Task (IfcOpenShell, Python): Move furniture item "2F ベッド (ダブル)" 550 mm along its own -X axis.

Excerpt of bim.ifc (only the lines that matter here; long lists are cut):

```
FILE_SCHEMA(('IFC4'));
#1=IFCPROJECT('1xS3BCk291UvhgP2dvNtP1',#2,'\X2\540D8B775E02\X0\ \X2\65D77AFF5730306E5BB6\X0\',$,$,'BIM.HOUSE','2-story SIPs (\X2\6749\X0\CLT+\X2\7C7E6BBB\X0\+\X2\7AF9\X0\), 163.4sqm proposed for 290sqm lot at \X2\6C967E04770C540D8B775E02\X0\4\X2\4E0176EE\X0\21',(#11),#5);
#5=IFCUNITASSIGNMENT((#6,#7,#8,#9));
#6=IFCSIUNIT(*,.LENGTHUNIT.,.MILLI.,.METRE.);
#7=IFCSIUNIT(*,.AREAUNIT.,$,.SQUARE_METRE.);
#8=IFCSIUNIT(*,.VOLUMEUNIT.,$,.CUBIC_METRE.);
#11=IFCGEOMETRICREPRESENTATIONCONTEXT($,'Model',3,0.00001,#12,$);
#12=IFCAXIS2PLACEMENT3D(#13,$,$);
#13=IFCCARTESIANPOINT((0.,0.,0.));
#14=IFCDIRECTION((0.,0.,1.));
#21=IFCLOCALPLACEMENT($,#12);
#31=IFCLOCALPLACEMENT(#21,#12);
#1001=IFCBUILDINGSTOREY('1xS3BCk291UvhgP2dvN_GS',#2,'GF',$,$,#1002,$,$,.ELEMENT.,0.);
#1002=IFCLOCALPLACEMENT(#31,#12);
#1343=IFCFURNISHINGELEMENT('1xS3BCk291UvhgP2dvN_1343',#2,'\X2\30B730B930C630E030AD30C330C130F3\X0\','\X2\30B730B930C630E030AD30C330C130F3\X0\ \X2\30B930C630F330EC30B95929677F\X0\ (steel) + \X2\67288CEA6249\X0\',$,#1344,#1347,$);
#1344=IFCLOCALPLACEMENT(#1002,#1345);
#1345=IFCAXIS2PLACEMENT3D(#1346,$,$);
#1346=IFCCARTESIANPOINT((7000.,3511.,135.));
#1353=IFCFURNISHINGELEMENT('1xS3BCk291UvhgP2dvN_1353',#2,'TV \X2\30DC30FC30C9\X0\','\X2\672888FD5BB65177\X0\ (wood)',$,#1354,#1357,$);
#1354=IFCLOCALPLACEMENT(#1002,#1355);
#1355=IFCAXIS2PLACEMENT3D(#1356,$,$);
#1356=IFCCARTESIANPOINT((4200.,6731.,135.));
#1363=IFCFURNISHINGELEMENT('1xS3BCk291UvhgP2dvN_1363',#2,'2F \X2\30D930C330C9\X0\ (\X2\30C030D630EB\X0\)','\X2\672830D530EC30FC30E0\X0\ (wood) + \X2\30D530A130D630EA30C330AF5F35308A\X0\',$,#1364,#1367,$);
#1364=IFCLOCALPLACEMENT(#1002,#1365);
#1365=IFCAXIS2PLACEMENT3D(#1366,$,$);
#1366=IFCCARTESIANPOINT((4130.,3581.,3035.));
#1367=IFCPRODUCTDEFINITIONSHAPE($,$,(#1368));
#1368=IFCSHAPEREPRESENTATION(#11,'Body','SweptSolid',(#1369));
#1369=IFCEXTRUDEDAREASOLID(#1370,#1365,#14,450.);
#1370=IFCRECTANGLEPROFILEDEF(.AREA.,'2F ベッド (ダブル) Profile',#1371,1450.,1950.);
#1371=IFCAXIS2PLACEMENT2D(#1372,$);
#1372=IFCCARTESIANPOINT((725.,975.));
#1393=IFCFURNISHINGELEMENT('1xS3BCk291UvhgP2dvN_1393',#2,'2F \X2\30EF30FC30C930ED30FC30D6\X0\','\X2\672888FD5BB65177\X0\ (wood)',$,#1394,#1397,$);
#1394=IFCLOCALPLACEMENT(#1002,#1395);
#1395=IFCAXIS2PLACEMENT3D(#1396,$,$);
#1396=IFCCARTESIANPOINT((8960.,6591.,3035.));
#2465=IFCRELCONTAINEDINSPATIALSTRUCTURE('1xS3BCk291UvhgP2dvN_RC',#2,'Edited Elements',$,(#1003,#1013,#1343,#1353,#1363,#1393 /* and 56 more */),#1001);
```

```python
import ifcopenshell
import ifcopenshell.api.geometry
import ifcopenshell.util.placement
import ifcopenshell.util.unit

model = ifcopenshell.open("bim.ifc")
unit_scale = ifcopenshell.util.unit.calculate_unit_scale(model)

item = model.by_id(1363)
matrix = ifcopenshell.util.placement.get_local_placement(item.ObjectPlacement)
matrix[:3, 3] -= matrix[:3, 0] * 0.55 / unit_scale
ifcopenshell.api.geometry.edit_object_placement(model, product=item, matrix=matrix, is_si=False)

print(ifcopenshell.util.placement.get_local_placement(item.ObjectPlacement).round(3) + 0.0)

model.write("bim-out.ifc")
```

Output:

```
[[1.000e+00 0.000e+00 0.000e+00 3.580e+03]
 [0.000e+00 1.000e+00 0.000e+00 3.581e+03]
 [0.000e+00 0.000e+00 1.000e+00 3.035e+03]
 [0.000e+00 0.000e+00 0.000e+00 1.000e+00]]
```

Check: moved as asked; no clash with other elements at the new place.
